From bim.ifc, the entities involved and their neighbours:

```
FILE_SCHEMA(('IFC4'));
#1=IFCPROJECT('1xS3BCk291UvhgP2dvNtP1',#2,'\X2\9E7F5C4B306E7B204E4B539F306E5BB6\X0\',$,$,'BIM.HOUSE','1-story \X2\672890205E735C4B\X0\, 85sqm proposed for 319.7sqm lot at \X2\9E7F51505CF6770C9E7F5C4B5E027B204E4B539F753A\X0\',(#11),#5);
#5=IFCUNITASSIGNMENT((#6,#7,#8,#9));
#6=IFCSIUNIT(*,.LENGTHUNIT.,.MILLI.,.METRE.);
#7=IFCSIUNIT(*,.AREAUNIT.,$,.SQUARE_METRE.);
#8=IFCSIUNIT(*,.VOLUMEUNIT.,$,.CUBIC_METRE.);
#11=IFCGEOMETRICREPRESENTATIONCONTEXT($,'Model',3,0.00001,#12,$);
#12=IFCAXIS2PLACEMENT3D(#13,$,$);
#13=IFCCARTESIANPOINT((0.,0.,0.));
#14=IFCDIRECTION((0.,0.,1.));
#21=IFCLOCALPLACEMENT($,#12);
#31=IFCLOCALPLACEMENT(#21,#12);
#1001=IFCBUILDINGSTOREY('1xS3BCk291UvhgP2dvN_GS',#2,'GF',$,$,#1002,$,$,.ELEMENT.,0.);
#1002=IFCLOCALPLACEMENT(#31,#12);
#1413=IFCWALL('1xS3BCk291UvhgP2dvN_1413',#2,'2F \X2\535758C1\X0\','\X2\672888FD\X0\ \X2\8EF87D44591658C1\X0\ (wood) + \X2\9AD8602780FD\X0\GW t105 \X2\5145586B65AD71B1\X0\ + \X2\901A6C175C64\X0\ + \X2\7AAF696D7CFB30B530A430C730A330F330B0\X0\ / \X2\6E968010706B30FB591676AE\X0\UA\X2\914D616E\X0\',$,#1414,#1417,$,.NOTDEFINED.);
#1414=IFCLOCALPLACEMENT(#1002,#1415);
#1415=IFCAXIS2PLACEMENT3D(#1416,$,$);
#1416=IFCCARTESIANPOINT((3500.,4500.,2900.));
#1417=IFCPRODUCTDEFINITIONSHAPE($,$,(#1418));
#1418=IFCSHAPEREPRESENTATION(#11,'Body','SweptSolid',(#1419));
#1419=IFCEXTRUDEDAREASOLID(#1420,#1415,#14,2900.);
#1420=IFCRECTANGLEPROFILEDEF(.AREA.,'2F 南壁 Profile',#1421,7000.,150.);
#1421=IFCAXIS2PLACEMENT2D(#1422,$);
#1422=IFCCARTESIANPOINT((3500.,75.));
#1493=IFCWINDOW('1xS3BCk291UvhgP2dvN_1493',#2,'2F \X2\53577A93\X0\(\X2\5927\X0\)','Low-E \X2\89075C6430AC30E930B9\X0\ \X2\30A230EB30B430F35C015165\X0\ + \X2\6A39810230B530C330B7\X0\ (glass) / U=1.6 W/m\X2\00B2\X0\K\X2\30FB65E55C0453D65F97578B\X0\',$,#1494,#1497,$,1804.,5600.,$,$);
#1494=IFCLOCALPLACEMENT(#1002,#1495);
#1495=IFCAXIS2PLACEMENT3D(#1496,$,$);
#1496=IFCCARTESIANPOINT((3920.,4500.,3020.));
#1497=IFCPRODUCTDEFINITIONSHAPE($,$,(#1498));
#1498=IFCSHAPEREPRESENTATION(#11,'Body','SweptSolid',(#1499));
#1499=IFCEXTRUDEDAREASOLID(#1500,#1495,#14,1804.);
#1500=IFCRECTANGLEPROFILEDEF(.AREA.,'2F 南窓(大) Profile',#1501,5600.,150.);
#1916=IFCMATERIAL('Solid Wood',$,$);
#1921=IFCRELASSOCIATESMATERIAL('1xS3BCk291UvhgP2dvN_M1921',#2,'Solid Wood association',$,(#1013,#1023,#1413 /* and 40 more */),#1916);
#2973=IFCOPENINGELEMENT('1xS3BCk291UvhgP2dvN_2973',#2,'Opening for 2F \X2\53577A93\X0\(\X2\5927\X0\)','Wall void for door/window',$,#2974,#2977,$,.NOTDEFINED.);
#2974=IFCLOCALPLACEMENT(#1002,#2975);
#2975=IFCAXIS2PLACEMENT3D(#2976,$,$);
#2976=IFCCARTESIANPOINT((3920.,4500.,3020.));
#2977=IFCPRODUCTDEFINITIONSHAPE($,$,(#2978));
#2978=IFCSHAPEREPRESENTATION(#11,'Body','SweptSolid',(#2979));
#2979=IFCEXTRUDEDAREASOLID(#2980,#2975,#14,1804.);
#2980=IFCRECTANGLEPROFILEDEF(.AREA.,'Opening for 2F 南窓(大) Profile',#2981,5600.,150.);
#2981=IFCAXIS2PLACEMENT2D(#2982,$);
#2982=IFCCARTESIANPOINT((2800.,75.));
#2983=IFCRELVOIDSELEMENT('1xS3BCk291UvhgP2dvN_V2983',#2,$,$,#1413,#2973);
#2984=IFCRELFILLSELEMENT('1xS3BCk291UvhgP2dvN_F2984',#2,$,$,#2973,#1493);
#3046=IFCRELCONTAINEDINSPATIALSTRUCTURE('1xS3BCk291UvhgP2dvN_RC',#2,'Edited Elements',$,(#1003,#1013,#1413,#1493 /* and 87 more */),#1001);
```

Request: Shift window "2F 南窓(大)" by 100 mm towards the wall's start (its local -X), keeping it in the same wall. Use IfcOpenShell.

```python
import ifcopenshell
import ifcopenshell.api.geometry
import ifcopenshell.util.placement

model = ifcopenshell.open("bim.ifc")

window = model.by_id(1493)
opening = window.FillsVoids[0].RelatingOpeningElement
wall = opening.VoidsElements[0].RelatingBuildingElement

wall_matrix = ifcopenshell.util.placement.get_local_placement(wall.ObjectPlacement)
shift = wall_matrix[:3, 0] * -100.0
before = ifcopenshell.util.placement.get_local_placement(window.ObjectPlacement)[:3, 3].copy()

# The window is not placed relative to its opening, so move both.
for product in (opening, window):
    matrix = ifcopenshell.util.placement.get_local_placement(product.ObjectPlacement)
    matrix[:3, 3] += shift
    ifcopenshell.api.geometry.edit_object_placement(model, product=product, matrix=matrix, is_si=False)

after = ifcopenshell.util.placement.get_local_placement(window.ObjectPlacement)[:3, 3]
print("window moved by", (after - before).round(3) + 0.0)

model.write("bim_updated.ifc")
```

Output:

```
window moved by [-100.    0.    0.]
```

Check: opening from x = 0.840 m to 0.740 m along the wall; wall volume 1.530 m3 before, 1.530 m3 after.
